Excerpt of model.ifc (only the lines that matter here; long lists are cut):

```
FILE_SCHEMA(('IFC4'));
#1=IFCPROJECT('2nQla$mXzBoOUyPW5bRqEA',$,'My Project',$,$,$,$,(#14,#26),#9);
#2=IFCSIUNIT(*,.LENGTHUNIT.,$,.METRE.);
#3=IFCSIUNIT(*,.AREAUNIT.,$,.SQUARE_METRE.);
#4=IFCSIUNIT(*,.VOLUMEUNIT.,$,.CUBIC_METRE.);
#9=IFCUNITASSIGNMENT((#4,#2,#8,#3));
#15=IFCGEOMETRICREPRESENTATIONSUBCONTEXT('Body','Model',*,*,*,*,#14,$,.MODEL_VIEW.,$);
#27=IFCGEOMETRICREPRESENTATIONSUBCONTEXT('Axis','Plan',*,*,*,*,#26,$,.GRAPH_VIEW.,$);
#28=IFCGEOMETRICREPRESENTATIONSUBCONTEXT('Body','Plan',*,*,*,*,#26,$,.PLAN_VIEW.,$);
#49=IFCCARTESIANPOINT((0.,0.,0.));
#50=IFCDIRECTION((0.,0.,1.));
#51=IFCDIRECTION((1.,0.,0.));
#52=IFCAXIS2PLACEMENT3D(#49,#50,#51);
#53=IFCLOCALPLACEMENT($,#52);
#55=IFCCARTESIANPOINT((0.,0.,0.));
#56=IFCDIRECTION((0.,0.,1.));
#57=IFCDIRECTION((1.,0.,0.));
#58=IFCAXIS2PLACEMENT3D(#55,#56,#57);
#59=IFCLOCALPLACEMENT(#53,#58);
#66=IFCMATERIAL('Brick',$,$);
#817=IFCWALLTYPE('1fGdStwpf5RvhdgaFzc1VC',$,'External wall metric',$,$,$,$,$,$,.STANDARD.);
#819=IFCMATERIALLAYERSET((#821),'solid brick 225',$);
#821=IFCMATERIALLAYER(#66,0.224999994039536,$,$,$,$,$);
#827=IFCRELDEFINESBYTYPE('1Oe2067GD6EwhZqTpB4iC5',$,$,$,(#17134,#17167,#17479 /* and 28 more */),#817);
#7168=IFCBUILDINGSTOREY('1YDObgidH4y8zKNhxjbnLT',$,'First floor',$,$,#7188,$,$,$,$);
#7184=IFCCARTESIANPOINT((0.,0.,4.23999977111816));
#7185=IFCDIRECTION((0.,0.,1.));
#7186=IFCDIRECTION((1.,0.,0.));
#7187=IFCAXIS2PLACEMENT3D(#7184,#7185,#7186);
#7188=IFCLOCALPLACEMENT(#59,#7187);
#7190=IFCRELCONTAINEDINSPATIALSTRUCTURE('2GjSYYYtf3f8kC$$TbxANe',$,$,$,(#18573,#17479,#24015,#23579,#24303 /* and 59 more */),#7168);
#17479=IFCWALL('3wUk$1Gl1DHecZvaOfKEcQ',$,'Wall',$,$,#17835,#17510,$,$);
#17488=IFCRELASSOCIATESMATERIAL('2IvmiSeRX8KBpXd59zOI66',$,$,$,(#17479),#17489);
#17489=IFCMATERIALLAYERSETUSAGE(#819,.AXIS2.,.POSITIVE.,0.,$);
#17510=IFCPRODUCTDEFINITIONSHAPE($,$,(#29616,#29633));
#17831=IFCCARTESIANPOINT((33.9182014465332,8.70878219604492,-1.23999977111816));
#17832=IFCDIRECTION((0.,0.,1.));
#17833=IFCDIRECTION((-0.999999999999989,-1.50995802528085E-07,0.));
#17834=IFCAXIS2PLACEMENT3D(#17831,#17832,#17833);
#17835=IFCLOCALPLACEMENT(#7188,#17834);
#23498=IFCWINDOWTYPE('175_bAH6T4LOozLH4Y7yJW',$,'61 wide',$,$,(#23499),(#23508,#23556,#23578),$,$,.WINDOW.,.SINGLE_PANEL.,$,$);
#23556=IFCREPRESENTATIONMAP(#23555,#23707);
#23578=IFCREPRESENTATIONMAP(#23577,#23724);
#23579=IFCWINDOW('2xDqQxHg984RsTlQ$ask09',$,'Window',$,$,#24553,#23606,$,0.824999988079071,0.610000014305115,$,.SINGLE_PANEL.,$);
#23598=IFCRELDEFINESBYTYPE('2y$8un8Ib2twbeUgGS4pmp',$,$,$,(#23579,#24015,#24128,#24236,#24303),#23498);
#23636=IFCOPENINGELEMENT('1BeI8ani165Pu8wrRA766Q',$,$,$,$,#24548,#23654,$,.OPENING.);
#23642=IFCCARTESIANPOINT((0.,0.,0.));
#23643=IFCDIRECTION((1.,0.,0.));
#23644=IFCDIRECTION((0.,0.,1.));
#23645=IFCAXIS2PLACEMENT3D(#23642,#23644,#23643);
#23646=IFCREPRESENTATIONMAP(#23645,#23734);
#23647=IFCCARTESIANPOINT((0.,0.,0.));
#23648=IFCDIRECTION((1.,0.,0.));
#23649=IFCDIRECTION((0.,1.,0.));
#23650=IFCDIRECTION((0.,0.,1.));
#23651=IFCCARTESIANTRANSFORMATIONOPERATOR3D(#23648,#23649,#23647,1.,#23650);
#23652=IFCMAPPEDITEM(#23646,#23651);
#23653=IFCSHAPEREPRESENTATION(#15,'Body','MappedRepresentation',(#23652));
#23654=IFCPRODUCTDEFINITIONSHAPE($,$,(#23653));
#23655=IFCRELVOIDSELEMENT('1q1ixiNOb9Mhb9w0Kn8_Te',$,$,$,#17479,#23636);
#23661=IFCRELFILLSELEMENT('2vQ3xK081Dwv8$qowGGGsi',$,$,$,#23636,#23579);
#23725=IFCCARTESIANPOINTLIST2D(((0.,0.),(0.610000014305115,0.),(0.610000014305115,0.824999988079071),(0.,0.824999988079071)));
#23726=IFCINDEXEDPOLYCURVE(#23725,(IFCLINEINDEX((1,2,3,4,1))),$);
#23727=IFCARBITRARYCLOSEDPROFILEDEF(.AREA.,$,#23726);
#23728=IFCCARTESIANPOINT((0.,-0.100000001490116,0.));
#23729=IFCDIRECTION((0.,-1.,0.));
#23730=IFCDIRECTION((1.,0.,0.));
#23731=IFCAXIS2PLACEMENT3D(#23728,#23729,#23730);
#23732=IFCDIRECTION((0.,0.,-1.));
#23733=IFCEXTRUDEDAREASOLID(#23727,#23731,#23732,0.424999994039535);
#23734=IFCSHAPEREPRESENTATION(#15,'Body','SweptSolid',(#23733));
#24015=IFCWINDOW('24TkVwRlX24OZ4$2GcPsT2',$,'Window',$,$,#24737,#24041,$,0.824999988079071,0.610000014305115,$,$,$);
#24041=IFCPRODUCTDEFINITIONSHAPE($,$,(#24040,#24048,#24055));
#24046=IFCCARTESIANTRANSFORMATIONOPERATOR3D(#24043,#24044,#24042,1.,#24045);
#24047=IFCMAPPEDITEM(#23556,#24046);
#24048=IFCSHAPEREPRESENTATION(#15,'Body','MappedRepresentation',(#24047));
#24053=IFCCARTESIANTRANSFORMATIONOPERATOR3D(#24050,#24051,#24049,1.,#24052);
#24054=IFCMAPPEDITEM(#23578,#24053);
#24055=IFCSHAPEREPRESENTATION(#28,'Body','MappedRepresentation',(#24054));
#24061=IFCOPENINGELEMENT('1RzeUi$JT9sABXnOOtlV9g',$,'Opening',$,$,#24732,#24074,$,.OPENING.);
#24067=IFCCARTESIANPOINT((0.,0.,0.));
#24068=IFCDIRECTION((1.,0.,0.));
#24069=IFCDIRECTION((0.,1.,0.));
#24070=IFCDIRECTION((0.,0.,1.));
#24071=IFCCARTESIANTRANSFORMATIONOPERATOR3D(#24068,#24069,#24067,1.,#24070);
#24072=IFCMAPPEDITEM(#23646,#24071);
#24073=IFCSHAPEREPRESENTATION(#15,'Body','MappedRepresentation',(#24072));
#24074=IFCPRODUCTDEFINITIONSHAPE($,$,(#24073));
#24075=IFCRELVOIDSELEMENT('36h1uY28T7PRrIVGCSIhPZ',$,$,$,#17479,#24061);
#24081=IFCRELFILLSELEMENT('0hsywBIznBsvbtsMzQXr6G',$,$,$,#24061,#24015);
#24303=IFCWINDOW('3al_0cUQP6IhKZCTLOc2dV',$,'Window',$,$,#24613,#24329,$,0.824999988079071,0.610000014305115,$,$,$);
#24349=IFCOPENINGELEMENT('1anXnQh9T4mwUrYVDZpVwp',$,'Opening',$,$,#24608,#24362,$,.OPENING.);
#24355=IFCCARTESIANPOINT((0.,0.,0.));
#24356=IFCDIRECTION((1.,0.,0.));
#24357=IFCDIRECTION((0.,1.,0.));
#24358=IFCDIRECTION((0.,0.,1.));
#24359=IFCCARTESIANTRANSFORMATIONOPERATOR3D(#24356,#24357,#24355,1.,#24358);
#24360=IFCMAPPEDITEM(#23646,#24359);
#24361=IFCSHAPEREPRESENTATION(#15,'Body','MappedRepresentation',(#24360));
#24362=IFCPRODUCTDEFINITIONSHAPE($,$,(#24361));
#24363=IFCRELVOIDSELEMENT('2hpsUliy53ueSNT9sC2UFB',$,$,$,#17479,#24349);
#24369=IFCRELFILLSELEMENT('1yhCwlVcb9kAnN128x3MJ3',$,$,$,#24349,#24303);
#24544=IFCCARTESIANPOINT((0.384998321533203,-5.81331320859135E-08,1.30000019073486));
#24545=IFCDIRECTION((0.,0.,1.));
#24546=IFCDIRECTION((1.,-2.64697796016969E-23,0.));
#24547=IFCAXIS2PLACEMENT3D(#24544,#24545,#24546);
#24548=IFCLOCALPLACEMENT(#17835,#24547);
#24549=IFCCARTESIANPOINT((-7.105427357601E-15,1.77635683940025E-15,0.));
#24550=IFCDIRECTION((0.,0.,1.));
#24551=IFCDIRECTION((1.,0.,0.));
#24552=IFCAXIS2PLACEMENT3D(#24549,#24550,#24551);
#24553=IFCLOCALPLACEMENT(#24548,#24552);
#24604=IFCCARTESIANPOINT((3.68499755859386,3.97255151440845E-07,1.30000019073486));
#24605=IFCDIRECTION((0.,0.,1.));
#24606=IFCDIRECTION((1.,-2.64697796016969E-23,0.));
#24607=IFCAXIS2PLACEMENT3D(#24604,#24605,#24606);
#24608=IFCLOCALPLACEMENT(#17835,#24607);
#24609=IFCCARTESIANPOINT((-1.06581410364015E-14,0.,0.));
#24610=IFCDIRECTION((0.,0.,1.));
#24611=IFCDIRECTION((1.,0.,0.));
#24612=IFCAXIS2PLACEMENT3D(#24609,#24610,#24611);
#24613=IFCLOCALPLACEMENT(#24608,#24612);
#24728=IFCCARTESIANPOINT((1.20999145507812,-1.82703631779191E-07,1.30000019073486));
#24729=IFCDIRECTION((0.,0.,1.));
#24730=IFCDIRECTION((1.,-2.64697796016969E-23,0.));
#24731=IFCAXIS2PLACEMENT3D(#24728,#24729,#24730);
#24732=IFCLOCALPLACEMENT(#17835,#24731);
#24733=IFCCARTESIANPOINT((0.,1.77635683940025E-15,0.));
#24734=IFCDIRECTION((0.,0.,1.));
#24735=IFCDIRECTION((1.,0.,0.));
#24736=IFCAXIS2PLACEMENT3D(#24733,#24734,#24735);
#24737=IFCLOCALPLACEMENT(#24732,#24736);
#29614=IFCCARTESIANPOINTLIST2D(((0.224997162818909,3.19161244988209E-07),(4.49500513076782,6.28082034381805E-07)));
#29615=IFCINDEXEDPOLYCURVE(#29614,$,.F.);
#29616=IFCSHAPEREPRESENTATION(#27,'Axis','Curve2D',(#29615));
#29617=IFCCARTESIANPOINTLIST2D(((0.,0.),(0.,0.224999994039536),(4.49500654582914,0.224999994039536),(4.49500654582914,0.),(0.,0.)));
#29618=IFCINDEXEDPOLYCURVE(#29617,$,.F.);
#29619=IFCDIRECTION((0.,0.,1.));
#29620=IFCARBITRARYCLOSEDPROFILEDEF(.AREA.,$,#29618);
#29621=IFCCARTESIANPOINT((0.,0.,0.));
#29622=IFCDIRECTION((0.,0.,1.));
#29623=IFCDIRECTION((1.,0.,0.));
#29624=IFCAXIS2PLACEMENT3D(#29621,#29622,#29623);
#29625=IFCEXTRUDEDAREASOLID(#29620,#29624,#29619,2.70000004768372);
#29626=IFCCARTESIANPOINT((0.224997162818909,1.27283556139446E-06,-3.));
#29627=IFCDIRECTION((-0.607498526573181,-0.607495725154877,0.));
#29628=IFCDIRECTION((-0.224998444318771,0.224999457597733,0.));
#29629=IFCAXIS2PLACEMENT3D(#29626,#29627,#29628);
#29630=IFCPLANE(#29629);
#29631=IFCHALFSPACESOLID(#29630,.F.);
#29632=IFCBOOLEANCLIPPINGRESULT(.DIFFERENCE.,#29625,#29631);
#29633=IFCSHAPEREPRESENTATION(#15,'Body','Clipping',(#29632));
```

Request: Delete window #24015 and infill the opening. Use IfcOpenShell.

```python
import ifcopenshell
import ifcopenshell.api.feature
import ifcopenshell.api.root
import ifcopenshell.geom
import ifcopenshell.util.shape

model = ifcopenshell.open("model.ifc")
settings = ifcopenshell.geom.settings()


def volume(element):
    """Net volume in cubic metres, openings subtracted."""
    shape = ifcopenshell.geom.create_shape(settings, element)
    return ifcopenshell.util.shape.get_volume(shape.geometry)


window = model.by_guid("24TkVwRlX24OZ4$2GcPsT2")
opening = window.FillsVoids[0].RelatingOpeningElement
wall = opening.VoidsElements[0].RelatingBuildingElement
before = volume(wall)

ifcopenshell.api.root.remove_product(model, product=window)
ifcopenshell.api.feature.remove_feature(model, feature=opening)

after = volume(wall)

print(f"wall volume {before:.3f} -> {after:.3f} m3")

model.write("model_updated.ifc")
```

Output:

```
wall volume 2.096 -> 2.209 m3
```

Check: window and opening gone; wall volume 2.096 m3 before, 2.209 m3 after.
